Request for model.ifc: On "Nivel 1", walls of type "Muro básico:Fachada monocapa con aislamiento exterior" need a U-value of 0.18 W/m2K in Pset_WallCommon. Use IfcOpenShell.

First a look at what the model holds.

```python
import ifcopenshell
import ifcopenshell.util.element

model = ifcopenshell.open("model.ifc")
print(model.schema)
storey = next(s for s in model.by_type("IfcBuildingStorey") if s.Name == "Nivel 1")
walls = [e for e in ifcopenshell.util.element.get_decomposition(storey) if e.is_a("IfcWall")]
seen = {}
for e in walls:
    element_type = ifcopenshell.util.element.get_type(e)
    key = (element_type.Name if element_type != e and element_type else None, ifcopenshell.util.element.get_pset(e, "Pset_WallCommon", "ThermalTransmittance"))
    seen[key] = seen.get(key, 0) + 1
for (name, value), count in sorted(seen.items(), key=str):
    print(count, "x", name, "|", value)
```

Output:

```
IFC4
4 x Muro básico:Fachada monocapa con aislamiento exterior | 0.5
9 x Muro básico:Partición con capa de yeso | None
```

```python
import ifcopenshell
import ifcopenshell.api.pset
import ifcopenshell.util.element

model = ifcopenshell.open("model.ifc")

storey = next(s for s in model.by_type("IfcBuildingStorey") if s.Name == "Nivel 1")
walls = [e for e in ifcopenshell.util.element.get_decomposition(storey) if e.is_a("IfcWall")]

count = 0
for e in walls:
    element_type = ifcopenshell.util.element.get_type(e)
    if element_type in (None, e) or element_type.Name != "Muro básico:Fachada monocapa con aislamiento exterior":
        continue
    # add_pset returns the element's existing set when there is one.
    pset = ifcopenshell.api.pset.add_pset(model, product=e, name="Pset_WallCommon")
    ifcopenshell.api.pset.edit_pset(model, pset=pset, properties={"ThermalTransmittance": 0.18})
    count += 1

print(count, "walls updated")

model.write("model_rev.ifc")
```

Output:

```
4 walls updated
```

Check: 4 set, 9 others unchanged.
